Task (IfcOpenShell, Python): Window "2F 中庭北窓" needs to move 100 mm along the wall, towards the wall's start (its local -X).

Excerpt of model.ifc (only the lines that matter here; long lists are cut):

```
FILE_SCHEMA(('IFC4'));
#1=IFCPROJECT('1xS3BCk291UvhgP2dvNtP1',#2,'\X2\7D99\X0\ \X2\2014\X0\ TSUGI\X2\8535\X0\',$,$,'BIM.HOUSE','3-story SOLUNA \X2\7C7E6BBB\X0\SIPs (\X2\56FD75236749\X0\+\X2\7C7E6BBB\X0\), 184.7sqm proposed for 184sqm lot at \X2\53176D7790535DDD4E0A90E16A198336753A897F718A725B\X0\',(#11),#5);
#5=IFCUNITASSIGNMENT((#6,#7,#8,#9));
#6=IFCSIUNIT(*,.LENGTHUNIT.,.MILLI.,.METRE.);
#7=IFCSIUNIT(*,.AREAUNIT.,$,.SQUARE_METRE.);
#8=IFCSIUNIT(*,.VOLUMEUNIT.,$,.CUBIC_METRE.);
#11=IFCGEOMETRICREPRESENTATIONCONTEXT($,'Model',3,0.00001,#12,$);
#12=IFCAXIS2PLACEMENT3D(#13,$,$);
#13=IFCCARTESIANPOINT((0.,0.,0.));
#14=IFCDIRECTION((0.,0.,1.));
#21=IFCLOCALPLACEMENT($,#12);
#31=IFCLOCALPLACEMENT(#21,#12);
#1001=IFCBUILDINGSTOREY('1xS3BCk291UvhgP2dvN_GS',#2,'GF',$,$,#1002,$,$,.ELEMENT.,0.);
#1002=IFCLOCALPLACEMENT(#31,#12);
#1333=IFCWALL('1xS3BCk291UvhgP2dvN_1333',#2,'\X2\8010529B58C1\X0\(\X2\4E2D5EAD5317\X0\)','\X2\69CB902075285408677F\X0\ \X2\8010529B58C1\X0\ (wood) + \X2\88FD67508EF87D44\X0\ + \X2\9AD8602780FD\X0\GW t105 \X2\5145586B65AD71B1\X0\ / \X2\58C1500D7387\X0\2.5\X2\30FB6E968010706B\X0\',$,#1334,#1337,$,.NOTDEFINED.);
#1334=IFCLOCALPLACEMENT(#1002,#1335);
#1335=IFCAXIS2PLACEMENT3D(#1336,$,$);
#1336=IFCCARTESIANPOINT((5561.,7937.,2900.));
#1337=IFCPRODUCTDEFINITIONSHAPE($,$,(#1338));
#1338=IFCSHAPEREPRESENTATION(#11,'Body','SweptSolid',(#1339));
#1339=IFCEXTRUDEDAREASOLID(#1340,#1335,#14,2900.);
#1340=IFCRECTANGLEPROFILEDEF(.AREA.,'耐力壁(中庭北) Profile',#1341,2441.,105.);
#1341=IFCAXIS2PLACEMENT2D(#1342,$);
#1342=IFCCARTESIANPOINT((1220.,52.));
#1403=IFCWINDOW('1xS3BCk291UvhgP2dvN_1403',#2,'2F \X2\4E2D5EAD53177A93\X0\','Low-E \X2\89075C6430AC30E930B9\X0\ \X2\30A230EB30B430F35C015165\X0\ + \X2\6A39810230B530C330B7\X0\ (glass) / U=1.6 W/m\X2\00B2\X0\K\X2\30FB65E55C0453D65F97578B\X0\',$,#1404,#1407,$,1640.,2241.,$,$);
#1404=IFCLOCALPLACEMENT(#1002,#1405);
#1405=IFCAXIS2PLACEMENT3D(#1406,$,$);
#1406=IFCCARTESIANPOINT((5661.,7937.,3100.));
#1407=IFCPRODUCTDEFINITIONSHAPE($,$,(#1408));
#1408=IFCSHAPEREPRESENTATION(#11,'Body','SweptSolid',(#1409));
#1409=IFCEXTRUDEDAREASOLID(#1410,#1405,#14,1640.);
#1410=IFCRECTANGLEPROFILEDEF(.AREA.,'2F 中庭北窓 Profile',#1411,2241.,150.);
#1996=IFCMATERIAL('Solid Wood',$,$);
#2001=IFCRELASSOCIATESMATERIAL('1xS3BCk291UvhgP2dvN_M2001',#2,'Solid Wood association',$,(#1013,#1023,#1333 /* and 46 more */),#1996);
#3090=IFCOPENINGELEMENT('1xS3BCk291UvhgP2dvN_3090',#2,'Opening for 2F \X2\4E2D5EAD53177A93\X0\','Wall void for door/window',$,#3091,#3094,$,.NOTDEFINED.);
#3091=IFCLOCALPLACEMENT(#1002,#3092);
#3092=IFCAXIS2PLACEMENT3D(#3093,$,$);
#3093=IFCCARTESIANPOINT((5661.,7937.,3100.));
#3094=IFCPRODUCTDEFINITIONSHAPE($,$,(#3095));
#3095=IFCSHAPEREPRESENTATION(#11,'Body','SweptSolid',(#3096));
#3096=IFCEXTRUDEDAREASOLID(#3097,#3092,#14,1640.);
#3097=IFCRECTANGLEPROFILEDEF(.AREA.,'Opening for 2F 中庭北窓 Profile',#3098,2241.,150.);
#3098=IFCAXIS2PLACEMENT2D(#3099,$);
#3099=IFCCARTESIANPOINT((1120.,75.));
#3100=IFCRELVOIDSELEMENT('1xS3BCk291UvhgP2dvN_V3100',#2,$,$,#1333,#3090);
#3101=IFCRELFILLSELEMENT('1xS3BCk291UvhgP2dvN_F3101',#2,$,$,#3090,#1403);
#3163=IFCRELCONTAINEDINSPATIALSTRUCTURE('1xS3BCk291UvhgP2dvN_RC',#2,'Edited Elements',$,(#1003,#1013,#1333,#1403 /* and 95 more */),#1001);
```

```python
import ifcopenshell
import ifcopenshell.api.geometry
import ifcopenshell.util.placement

model = ifcopenshell.open("model.ifc")

window = model.by_guid("1xS3BCk291UvhgP2dvN_1403")
opening = window.FillsVoids[0].RelatingOpeningElement
wall = opening.VoidsElements[0].RelatingBuildingElement

wall_matrix = ifcopenshell.util.placement.get_local_placement(wall.ObjectPlacement)
shift = wall_matrix[:3, 0] * -100.0
before = ifcopenshell.util.placement.get_local_placement(window.ObjectPlacement)[:3, 3].copy()

# The window is not placed relative to its opening, so move both.
for product in (opening, window):
    matrix = ifcopenshell.util.placement.get_local_placement(product.ObjectPlacement)
    matrix[:3, 3] += shift
    ifcopenshell.api.geometry.edit_object_placement(model, product=product, matrix=matrix, is_si=False)

after = ifcopenshell.util.placement.get_local_placement(window.ObjectPlacement)[:3, 3]
print("window moved by", (after - before).round(3) + 0.0)

model.write("model_updated.ifc")
```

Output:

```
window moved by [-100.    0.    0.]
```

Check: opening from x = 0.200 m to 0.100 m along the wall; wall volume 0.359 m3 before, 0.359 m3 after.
